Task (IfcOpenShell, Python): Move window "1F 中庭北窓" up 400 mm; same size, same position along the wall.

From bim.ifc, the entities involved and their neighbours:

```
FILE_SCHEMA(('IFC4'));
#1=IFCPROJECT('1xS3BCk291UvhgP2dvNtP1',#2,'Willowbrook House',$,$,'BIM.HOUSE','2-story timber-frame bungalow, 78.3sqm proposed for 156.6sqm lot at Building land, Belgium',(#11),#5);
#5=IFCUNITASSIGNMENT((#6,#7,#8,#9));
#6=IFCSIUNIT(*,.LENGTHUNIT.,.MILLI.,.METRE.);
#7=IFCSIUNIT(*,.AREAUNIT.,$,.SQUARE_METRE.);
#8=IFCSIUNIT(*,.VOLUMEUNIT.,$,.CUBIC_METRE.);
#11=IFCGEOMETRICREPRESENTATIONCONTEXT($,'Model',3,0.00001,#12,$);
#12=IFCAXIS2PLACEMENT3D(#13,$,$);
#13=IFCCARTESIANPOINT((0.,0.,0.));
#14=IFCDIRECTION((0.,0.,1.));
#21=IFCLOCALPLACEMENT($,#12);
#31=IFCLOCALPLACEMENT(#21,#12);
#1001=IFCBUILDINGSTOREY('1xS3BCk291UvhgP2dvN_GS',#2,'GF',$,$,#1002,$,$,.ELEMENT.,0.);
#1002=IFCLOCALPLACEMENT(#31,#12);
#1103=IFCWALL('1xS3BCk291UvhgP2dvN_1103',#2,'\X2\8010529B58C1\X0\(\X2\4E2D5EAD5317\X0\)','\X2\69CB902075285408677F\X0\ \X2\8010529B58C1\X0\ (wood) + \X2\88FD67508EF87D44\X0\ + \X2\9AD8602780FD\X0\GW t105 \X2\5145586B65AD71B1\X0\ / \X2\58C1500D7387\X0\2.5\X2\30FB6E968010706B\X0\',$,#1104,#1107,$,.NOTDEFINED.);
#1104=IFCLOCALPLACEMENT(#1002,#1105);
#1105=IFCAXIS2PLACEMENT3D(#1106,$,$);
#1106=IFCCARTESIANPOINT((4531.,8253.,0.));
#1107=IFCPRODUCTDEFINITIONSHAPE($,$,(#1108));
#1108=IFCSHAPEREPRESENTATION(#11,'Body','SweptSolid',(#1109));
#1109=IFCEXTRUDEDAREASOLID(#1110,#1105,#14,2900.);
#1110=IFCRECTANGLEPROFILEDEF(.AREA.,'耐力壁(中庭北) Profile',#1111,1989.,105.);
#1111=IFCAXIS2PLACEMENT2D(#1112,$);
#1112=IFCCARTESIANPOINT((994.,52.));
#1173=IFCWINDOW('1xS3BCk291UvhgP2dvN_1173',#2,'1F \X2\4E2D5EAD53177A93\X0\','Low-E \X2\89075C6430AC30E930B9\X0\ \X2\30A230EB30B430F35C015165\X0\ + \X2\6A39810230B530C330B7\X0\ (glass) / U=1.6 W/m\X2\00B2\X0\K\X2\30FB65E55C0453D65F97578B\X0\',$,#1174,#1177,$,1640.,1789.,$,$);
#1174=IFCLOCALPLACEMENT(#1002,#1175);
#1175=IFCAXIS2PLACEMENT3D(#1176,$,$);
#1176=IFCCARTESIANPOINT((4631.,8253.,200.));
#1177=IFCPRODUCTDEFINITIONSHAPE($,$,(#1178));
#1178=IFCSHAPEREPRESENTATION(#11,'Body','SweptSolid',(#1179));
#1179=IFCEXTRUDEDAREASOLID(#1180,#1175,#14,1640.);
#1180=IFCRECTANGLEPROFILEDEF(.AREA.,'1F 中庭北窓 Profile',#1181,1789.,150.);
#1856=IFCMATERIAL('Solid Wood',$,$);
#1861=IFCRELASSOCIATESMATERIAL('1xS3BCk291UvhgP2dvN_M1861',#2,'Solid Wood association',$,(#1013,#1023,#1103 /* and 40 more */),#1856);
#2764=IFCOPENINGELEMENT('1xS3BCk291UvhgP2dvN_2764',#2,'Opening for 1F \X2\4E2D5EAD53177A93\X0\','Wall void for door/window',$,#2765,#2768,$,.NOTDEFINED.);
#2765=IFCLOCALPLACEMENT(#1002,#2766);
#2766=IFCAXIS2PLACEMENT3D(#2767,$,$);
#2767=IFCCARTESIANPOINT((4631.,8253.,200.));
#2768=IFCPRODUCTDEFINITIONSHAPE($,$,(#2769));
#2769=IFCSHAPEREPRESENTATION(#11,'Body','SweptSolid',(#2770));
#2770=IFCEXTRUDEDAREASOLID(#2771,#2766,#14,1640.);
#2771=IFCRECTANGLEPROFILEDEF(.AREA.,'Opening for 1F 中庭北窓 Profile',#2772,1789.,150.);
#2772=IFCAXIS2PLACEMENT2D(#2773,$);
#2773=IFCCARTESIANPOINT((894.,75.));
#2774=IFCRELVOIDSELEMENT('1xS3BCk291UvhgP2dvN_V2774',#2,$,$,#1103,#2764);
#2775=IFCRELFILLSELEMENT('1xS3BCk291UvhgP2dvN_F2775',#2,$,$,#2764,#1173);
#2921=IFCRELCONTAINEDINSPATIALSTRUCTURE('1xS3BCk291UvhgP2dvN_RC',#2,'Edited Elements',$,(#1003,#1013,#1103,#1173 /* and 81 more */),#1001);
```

```python
import numpy as np
import ifcopenshell
import ifcopenshell.api.geometry
import ifcopenshell.util.placement
import ifcopenshell.util.unit

model = ifcopenshell.open("bim.ifc")
unit_scale = ifcopenshell.util.unit.calculate_unit_scale(model)

window = model.by_id(1173)
opening = window.FillsVoids[0].RelatingOpeningElement
dz = 0.4 / unit_scale

shift = np.array([0.0, 0.0, dz])
# The window is not placed relative to its opening, so move both.
for product in (opening, window):
    matrix = ifcopenshell.util.placement.get_local_placement(product.ObjectPlacement)
    matrix[:3, 3] += shift
    ifcopenshell.api.geometry.edit_object_placement(model, product=product, matrix=matrix, is_si=False)

print(f"moved by {dz * unit_scale:+.3f} m")

model.write("bim-out.ifc")
```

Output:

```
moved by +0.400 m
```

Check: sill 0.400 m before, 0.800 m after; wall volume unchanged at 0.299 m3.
